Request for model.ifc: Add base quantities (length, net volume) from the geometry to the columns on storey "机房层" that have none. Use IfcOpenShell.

First a look at what the model holds.

```python
import ifcopenshell
import ifcopenshell.util.element
import ifcopenshell.util.unit

model = ifcopenshell.open("model.ifc")
print(model.schema)
for unit_type in ("LENGTHUNIT", "AREAUNIT", "VOLUMEUNIT"):
    print(unit_type, ifcopenshell.util.unit.calculate_unit_scale(model, unit_type))
storey = next(s for s in model.by_type("IfcBuildingStorey") if s.Name == "机房层")
columns = [e for e in ifcopenshell.util.element.get_decomposition(storey) if e.is_a("IfcColumn")]
for e in sorted(columns, key=lambda e: e.id()):
    print(e.id(), e.is_a(), e.Name, list(ifcopenshell.util.element.get_psets(e, qtos_only=True)), sep=" | ")
```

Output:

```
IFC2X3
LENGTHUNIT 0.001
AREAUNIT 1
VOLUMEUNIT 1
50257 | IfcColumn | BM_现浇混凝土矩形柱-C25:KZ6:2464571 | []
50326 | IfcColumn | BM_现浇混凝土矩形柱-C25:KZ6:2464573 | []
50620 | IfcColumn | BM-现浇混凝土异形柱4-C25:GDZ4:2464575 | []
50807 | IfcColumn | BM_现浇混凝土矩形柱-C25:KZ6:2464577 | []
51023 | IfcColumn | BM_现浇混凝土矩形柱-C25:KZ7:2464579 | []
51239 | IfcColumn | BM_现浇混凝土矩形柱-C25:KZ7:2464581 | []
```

```python
import ifcopenshell
import ifcopenshell.api.pset
import ifcopenshell.geom
import ifcopenshell.util.element
import ifcopenshell.util.shape
import ifcopenshell.util.unit

model = ifcopenshell.open("model.ifc")
unit_scale = ifcopenshell.util.unit.calculate_unit_scale(model)
volume_scale = ifcopenshell.util.unit.calculate_unit_scale(model, "VOLUMEUNIT")
settings = ifcopenshell.geom.settings()

storey = next(s for s in model.by_type("IfcBuildingStorey") if s.Name == "机房层")
columns = [e for e in ifcopenshell.util.element.get_decomposition(storey) if e.is_a("IfcColumn")]

for e in sorted(columns, key=lambda e: e.id()):
    if ifcopenshell.util.element.get_psets(e, qtos_only=True, should_inherit=False):
        continue
    # Geometry comes back in metres, in the element's own axes.
    shape = ifcopenshell.geom.create_shape(settings, e)
    values = {
        "Length": ifcopenshell.util.shape.get_z(shape.geometry) / unit_scale,
        "NetVolume": ifcopenshell.util.shape.get_volume(shape.geometry) / volume_scale,
    }
    qto = ifcopenshell.api.pset.add_qto(model, product=e, name="BaseQuantities")
    ifcopenshell.api.pset.edit_qto(model, qto=qto, properties=values)
    print(e.id(), {k: round(v, 3) for k, v in values.items()})

model.write("model_rev.ifc")
```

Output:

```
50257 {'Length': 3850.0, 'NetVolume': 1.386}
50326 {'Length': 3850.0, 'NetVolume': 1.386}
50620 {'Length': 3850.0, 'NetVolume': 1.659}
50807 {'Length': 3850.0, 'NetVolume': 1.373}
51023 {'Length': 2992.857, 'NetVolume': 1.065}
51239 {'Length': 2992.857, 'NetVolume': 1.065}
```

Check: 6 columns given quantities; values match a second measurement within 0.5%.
